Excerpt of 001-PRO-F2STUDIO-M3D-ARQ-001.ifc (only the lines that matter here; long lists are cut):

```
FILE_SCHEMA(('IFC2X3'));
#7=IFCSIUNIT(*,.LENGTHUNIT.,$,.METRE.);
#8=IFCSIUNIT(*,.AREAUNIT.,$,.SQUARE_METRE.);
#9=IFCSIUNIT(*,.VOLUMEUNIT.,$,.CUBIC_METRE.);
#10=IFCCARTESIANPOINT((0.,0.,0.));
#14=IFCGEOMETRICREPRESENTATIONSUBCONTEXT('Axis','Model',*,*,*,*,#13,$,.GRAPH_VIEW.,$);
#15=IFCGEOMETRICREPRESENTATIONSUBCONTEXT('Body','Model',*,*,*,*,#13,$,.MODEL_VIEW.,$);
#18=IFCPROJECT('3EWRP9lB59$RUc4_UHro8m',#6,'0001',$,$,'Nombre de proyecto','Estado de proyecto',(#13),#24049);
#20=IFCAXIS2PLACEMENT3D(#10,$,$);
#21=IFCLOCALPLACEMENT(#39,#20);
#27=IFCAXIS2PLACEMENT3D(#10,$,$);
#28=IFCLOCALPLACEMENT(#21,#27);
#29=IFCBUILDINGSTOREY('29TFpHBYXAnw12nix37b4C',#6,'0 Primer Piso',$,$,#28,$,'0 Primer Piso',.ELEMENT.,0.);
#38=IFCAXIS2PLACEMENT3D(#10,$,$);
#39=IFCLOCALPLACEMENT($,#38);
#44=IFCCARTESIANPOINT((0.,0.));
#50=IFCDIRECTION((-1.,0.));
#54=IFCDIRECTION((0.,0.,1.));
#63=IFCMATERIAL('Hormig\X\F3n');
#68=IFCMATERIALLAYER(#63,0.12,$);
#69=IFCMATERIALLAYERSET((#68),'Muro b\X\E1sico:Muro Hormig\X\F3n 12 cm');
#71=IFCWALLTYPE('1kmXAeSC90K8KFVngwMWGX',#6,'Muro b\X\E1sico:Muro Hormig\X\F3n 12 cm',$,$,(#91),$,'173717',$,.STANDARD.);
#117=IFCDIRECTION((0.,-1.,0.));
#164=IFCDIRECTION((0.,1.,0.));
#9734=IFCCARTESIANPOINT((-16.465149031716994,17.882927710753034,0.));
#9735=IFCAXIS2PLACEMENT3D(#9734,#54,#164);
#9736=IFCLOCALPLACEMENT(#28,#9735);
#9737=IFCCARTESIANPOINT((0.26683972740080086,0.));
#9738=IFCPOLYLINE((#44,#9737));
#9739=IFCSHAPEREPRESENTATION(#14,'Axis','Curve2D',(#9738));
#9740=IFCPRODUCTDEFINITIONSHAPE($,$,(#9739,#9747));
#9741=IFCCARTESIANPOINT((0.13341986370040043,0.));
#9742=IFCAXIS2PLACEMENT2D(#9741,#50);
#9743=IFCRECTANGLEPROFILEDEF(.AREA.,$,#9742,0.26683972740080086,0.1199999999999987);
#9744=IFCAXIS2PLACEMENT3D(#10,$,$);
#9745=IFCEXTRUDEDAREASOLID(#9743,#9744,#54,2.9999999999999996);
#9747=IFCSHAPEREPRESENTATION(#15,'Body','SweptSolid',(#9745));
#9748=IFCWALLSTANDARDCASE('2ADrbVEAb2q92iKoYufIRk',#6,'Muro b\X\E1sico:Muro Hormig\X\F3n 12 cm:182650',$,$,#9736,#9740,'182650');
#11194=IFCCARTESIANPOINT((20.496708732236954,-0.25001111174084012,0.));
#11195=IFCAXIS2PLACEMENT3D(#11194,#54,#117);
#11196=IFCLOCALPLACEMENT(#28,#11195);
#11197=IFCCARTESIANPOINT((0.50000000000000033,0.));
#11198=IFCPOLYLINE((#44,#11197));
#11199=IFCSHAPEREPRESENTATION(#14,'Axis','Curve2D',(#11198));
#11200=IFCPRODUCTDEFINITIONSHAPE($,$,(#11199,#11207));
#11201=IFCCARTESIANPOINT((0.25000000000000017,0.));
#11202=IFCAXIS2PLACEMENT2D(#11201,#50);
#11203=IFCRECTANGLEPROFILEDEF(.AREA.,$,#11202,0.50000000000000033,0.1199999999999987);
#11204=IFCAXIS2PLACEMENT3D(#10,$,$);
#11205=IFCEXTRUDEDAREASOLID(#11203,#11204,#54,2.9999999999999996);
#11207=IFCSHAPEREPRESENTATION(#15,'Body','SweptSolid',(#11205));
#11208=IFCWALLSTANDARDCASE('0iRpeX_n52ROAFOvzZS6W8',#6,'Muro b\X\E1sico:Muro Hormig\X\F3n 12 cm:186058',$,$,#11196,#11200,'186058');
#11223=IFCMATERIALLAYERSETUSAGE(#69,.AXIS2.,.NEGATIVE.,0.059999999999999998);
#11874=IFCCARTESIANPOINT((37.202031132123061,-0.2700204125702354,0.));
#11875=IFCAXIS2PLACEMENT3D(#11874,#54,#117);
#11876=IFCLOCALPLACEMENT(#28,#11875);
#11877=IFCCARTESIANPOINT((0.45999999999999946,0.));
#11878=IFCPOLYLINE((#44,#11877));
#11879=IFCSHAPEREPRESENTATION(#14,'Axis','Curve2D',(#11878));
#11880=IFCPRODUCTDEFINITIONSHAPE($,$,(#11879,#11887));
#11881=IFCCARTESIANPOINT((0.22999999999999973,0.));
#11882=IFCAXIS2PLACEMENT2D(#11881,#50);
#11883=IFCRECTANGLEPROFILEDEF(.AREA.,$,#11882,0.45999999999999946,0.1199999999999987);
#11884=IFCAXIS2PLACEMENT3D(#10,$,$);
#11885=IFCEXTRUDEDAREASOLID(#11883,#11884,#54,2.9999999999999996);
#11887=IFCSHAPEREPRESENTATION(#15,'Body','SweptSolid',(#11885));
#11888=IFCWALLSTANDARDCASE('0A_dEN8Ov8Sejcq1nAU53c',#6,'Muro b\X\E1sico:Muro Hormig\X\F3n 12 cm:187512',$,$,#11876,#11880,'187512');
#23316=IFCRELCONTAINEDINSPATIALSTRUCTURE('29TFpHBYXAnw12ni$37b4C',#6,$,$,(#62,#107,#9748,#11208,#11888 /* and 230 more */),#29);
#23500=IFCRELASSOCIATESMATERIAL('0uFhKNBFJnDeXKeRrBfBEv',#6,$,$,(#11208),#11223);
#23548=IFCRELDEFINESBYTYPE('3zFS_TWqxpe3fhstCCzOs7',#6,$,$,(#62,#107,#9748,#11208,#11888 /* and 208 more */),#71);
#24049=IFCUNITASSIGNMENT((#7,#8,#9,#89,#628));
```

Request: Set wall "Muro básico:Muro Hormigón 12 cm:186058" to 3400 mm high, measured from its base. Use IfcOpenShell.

```python
import ifcopenshell
import ifcopenshell.geom
import ifcopenshell.util.representation
import ifcopenshell.util.shape
import ifcopenshell.util.unit

model = ifcopenshell.open("001-PRO-F2STUDIO-M3D-ARQ-001.ifc")
unit_scale = ifcopenshell.util.unit.calculate_unit_scale(model)
settings = ifcopenshell.geom.settings()


def volume(element):
    """Net volume in cubic metres, openings subtracted."""
    shape = ifcopenshell.geom.create_shape(settings, element)
    return ifcopenshell.util.shape.get_volume(shape.geometry)


wall = model.by_guid("0iRpeX_n52ROAFOvzZS6W8")
before = volume(wall)

body = ifcopenshell.util.representation.get_representation(wall, "Model", "Body")
solid = body.Items[0]
old_height = solid.Depth
solid.Depth = 3.4 / unit_scale
after = volume(wall)

print(f"height {old_height:g} -> {solid.Depth:g}, volume {before:.3f} -> {after:.3f} m3")

model.write("001-PRO-F2STUDIO-M3D-ARQ-001_updated.ifc")
```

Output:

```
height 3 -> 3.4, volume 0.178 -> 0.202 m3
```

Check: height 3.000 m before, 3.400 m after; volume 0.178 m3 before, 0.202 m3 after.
